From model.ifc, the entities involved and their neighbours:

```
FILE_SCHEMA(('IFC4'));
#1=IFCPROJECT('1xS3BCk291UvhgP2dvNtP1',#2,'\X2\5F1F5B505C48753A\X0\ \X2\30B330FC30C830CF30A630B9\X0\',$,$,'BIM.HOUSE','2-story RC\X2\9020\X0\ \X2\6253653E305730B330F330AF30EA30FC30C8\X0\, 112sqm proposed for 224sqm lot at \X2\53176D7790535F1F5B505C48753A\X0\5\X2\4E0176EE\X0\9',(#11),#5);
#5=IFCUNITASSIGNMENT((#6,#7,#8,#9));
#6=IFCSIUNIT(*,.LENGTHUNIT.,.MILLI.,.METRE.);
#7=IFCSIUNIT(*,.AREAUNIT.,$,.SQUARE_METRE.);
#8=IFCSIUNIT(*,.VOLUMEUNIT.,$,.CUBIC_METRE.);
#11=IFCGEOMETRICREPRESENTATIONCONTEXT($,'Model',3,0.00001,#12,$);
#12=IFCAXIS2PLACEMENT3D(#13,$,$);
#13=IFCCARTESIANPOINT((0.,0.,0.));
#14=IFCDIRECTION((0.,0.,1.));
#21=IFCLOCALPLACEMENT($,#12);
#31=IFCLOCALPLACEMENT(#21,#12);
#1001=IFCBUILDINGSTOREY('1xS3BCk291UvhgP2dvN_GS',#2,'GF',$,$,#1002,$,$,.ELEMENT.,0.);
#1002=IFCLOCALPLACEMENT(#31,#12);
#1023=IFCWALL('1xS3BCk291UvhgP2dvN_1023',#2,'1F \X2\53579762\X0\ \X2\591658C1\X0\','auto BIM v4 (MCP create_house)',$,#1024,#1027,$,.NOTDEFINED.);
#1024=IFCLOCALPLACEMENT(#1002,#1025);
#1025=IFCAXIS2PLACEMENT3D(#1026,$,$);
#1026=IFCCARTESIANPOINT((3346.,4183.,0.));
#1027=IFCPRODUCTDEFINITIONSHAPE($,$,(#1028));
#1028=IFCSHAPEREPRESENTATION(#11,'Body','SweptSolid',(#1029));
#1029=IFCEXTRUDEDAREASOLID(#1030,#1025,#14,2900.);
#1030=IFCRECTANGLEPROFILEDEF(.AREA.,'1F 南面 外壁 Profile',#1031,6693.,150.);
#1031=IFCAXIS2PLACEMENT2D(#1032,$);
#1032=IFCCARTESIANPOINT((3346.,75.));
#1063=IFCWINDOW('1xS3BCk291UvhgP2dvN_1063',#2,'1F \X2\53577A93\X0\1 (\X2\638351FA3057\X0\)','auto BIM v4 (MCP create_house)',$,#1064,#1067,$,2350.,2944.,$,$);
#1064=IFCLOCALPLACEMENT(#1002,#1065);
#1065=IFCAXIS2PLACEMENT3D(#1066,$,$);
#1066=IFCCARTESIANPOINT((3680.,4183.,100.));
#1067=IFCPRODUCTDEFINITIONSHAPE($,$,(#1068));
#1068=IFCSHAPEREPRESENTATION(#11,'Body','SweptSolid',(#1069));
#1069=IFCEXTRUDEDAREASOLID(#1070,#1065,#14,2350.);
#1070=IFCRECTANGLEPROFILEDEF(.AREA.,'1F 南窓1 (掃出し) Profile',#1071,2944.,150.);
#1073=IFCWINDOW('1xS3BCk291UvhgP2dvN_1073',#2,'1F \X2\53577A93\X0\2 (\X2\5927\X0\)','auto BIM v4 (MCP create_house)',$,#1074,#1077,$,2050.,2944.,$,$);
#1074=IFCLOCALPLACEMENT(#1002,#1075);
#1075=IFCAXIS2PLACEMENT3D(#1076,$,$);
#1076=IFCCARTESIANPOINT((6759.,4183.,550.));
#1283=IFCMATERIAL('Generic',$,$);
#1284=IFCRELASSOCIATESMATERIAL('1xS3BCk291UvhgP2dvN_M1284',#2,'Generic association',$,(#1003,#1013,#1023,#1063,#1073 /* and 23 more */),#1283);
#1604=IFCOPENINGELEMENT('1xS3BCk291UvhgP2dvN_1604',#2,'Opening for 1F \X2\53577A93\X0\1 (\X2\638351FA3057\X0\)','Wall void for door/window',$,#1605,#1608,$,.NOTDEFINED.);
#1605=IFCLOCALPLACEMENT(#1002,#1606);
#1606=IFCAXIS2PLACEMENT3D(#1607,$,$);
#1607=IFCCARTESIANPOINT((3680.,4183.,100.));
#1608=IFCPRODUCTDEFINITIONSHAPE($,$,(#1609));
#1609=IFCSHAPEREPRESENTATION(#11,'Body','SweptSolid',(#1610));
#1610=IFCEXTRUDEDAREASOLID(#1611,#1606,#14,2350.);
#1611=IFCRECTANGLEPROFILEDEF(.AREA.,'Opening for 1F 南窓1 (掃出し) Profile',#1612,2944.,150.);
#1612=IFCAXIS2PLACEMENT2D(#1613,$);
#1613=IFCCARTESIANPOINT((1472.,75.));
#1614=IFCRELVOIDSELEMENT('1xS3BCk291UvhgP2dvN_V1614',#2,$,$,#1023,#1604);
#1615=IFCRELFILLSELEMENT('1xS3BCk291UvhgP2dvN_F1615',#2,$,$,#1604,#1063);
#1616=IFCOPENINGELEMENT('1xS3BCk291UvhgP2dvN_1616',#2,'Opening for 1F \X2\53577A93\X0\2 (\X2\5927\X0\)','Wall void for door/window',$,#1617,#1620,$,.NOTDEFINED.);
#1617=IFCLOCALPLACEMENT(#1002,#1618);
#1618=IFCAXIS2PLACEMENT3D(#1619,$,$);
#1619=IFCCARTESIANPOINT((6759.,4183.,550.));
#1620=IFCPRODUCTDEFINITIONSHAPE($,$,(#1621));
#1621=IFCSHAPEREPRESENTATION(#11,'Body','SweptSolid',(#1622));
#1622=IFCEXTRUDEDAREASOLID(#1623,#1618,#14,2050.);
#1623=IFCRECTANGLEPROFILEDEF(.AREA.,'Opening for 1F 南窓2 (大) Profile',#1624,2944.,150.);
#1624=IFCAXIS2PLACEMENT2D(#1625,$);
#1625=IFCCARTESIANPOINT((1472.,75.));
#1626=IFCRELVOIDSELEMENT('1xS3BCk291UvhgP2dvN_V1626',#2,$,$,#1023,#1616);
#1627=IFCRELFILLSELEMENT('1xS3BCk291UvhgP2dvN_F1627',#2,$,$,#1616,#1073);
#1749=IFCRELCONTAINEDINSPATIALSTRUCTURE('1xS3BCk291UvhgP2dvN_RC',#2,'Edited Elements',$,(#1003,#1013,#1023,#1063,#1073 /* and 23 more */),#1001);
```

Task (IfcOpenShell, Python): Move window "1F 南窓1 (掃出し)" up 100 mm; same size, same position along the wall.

```python
import numpy as np
import ifcopenshell
import ifcopenshell.api.geometry
import ifcopenshell.util.placement
import ifcopenshell.util.unit

model = ifcopenshell.open("model.ifc")
unit_scale = ifcopenshell.util.unit.calculate_unit_scale(model)

window = model.by_guid("1xS3BCk291UvhgP2dvN_1063")
opening = window.FillsVoids[0].RelatingOpeningElement
dz = 0.1 / unit_scale

shift = np.array([0.0, 0.0, dz])
# The window is not placed relative to its opening, so move both.
for product in (opening, window):
    matrix = ifcopenshell.util.placement.get_local_placement(product.ObjectPlacement)
    matrix[:3, 3] += shift
    ifcopenshell.api.geometry.edit_object_placement(model, product=product, matrix=matrix, is_si=False)

print(f"moved by {dz * unit_scale:+.3f} m")

model.write("model-out.ifc")
```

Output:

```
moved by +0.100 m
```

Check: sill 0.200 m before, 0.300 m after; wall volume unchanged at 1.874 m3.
